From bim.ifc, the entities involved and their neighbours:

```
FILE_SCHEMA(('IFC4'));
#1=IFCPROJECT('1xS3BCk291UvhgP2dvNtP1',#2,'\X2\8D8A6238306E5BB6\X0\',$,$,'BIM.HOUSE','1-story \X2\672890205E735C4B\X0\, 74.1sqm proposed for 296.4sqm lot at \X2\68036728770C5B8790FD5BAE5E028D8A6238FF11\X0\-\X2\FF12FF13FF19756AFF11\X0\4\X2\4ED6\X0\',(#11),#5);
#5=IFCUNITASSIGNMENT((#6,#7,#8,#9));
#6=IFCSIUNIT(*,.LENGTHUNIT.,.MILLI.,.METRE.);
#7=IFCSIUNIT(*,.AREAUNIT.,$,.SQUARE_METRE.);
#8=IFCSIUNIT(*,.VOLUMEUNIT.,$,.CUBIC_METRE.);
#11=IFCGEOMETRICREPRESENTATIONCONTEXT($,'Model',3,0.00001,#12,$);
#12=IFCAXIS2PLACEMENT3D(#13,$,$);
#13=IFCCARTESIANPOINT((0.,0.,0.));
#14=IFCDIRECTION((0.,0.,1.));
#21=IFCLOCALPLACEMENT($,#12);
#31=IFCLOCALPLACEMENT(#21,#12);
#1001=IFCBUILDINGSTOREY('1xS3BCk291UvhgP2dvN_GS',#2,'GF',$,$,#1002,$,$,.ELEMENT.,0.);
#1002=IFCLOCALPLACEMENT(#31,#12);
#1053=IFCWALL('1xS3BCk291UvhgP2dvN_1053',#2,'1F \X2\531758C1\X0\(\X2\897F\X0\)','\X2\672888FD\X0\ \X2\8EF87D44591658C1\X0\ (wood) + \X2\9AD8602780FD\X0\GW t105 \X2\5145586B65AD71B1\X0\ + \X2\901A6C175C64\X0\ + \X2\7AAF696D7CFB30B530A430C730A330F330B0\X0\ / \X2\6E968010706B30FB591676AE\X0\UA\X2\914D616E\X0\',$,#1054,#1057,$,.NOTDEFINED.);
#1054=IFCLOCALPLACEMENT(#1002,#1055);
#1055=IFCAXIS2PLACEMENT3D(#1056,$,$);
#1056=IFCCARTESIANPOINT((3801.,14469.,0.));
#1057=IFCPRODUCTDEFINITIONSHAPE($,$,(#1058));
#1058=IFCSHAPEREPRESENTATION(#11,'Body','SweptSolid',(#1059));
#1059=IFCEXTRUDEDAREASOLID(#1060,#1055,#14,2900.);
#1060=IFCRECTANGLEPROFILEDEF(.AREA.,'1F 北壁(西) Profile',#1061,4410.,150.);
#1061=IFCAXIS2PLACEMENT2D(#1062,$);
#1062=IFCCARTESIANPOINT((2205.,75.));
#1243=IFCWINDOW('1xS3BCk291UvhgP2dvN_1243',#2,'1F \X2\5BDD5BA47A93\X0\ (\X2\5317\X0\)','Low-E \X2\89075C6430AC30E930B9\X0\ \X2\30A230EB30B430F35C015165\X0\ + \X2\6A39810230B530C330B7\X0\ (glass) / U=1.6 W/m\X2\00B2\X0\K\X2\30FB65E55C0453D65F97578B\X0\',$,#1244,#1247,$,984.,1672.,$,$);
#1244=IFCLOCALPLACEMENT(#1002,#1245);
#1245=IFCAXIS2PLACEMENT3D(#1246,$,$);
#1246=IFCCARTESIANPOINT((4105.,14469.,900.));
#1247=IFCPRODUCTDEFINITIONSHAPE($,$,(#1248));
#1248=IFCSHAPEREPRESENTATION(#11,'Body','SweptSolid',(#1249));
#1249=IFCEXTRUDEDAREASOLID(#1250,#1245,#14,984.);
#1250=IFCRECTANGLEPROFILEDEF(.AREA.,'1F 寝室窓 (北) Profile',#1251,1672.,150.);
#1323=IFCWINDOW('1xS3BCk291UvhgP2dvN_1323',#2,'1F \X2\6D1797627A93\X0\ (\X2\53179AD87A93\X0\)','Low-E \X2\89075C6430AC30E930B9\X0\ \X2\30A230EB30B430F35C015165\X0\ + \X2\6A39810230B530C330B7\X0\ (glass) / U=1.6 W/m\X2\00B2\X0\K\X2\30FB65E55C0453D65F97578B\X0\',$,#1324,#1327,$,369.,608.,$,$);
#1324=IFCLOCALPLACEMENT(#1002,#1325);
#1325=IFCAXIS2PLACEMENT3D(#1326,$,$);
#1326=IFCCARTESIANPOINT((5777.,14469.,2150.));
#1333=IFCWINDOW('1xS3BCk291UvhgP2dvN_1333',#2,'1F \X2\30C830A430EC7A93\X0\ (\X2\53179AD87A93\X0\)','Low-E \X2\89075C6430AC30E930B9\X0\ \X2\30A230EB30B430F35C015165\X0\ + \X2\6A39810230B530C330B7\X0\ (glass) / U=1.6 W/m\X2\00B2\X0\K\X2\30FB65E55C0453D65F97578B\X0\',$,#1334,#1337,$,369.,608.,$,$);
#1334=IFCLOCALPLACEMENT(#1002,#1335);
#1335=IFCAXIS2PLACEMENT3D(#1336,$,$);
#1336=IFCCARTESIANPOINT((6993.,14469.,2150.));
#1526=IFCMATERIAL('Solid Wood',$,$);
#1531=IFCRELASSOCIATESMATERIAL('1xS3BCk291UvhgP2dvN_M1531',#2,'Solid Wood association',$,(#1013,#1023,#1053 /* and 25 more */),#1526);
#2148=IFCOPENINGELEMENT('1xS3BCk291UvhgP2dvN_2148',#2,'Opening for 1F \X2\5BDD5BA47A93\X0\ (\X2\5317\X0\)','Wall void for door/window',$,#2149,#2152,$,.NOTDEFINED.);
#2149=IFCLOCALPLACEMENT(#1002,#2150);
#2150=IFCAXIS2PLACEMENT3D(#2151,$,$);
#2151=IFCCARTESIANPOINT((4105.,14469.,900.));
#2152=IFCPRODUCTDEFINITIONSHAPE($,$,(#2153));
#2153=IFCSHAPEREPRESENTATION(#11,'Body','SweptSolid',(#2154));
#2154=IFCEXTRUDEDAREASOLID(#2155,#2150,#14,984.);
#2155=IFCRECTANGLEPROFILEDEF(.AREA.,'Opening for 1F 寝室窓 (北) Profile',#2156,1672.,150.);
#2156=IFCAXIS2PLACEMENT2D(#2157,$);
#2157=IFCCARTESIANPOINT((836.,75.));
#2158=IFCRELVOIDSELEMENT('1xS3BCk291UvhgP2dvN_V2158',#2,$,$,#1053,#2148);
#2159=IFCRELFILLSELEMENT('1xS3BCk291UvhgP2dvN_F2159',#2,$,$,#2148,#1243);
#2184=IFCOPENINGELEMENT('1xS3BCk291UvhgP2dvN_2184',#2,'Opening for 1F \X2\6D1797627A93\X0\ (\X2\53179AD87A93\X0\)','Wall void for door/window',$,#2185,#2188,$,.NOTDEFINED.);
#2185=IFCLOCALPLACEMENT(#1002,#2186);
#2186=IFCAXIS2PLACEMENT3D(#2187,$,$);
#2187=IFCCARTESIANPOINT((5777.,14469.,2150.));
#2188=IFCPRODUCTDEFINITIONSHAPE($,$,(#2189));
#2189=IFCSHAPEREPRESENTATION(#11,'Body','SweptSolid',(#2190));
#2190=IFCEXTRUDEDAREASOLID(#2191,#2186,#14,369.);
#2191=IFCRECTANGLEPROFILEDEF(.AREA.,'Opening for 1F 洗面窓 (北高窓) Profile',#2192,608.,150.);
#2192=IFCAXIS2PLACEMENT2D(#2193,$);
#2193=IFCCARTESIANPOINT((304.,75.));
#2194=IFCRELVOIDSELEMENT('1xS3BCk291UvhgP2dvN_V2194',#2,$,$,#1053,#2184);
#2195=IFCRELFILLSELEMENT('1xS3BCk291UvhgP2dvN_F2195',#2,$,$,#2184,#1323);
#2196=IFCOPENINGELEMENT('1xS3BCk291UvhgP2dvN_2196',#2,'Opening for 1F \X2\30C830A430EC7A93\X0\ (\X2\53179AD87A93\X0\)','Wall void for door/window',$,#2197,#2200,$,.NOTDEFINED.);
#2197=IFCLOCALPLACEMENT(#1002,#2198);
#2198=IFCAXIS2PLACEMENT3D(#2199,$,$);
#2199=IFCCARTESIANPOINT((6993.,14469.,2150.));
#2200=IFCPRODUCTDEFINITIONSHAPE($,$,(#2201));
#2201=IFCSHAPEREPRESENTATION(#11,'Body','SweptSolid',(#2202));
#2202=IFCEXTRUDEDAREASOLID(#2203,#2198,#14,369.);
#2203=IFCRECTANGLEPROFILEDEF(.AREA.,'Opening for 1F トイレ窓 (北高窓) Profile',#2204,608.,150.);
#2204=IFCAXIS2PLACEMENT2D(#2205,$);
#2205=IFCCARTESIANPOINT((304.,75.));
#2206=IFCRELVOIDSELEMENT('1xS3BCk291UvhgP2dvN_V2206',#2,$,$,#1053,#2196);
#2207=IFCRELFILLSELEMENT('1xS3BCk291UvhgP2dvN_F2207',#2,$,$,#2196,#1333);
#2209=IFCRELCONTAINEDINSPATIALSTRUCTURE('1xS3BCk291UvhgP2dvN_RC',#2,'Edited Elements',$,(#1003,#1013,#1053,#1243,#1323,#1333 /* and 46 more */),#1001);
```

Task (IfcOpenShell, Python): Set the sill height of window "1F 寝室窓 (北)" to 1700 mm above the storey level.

```python
import numpy as np
import ifcopenshell
import ifcopenshell.api.geometry
import ifcopenshell.geom
import ifcopenshell.util.element
import ifcopenshell.util.placement
import ifcopenshell.util.shape
import ifcopenshell.util.unit

model = ifcopenshell.open("bim.ifc")
unit_scale = ifcopenshell.util.unit.calculate_unit_scale(model)

window = model.by_id(1243)
opening = window.FillsVoids[0].RelatingOpeningElement
storey = ifcopenshell.util.element.get_container(window, ifc_class="IfcBuildingStorey")
level = ifcopenshell.util.placement.get_local_placement(storey.ObjectPlacement)[2, 3]

# The opening's origin need not be at the sill, so measure its lowest point.
shape = ifcopenshell.geom.create_shape(ifcopenshell.geom.settings(), opening)
bottom = ifcopenshell.util.shape.get_shape_bottom_elevation(shape, shape.geometry) / unit_scale
dz = level + 1.7 / unit_scale - bottom

shift = np.array([0.0, 0.0, dz])
# The window is not placed relative to its opening, so move both.
for product in (opening, window):
    matrix = ifcopenshell.util.placement.get_local_placement(product.ObjectPlacement)
    matrix[:3, 3] += shift
    ifcopenshell.api.geometry.edit_object_placement(model, product=product, matrix=matrix, is_si=False)

print(f"moved by {dz * unit_scale:+.3f} m")

model.write("bim_rev.ifc")
```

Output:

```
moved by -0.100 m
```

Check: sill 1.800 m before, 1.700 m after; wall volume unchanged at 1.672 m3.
